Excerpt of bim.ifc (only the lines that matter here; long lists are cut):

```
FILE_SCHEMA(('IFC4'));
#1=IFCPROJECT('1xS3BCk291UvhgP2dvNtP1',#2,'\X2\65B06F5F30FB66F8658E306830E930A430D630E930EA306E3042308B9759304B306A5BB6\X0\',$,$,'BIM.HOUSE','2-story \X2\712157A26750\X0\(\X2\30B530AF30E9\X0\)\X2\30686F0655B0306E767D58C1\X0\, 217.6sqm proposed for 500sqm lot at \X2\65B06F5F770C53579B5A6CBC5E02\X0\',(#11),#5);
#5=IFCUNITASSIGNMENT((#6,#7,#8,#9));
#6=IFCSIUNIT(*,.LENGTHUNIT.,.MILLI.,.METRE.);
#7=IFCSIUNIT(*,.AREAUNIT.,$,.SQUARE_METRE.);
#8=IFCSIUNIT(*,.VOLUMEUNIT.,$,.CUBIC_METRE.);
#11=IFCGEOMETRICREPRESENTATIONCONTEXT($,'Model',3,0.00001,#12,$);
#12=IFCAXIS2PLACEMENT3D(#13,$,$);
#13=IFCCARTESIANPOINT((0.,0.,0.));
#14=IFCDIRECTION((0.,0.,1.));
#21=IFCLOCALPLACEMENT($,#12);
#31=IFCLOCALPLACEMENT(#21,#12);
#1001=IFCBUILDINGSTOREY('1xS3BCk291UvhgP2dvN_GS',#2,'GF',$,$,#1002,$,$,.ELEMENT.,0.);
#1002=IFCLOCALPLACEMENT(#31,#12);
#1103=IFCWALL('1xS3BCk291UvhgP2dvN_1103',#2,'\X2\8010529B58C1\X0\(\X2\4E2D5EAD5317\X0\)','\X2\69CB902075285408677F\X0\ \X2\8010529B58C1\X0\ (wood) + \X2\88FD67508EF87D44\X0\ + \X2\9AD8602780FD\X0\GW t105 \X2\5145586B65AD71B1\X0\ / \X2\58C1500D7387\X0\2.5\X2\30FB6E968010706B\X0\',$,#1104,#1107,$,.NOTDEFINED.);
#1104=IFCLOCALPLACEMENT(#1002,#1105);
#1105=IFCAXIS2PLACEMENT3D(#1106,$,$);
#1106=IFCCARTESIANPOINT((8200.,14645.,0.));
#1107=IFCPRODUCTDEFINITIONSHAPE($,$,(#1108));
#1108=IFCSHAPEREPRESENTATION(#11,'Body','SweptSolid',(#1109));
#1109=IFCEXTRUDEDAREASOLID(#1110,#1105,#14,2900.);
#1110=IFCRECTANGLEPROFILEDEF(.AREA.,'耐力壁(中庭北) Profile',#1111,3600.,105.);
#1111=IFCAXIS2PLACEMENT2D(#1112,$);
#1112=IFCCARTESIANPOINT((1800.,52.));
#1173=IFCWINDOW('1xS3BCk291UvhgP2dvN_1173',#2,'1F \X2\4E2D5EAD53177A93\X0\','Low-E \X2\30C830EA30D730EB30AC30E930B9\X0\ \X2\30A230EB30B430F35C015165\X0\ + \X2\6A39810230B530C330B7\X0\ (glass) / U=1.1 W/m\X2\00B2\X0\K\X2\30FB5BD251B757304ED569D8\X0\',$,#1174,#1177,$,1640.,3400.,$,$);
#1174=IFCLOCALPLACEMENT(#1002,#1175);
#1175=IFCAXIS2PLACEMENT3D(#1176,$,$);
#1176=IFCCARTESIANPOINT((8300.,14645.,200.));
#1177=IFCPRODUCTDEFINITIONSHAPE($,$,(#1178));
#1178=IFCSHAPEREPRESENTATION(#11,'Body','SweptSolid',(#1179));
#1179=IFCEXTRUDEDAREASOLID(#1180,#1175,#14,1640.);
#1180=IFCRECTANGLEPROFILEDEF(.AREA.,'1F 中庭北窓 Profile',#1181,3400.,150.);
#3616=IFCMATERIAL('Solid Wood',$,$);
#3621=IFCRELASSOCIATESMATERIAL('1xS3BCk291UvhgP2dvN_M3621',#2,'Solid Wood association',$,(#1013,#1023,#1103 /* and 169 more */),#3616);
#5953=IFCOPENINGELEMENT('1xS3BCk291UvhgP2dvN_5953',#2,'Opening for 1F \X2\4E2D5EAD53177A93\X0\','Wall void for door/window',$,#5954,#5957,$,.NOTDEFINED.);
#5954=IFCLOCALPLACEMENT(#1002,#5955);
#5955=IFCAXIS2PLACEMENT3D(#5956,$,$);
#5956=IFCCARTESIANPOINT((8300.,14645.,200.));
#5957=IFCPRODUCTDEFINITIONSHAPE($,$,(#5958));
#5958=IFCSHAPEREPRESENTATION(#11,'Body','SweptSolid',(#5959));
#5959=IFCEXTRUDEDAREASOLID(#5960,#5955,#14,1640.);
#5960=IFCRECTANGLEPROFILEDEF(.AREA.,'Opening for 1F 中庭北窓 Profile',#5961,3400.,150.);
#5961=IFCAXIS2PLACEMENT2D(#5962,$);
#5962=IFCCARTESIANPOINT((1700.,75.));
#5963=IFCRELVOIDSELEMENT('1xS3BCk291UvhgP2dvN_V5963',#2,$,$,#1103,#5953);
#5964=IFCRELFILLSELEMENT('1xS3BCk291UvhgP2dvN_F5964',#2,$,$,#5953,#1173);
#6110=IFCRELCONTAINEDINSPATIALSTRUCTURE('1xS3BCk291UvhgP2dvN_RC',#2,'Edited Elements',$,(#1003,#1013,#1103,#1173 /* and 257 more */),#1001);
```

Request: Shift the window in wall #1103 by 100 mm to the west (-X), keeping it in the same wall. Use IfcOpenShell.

```python
import ifcopenshell
import ifcopenshell.api.geometry
import ifcopenshell.util.placement
import ifcopenshell.util.unit

model = ifcopenshell.open("bim.ifc")
unit_scale = ifcopenshell.util.unit.calculate_unit_scale(model)

window = model.by_id(1173)
opening = window.FillsVoids[0].RelatingOpeningElement
wall = opening.VoidsElements[0].RelatingBuildingElement

wall_matrix = ifcopenshell.util.placement.get_local_placement(wall.ObjectPlacement)
shift = wall_matrix[:3, 0] * -0.1 / unit_scale
before = ifcopenshell.util.placement.get_local_placement(window.ObjectPlacement)[:3, 3].copy()

# The window is not placed relative to its opening, so move both.
for product in (opening, window):
    matrix = ifcopenshell.util.placement.get_local_placement(product.ObjectPlacement)
    matrix[:3, 3] += shift
    ifcopenshell.api.geometry.edit_object_placement(model, product=product, matrix=matrix, is_si=False)

after = ifcopenshell.util.placement.get_local_placement(window.ObjectPlacement)[:3, 3]
print("window moved by", (after - before).round(3) + 0.0)

model.write("bim_v2.ifc")
```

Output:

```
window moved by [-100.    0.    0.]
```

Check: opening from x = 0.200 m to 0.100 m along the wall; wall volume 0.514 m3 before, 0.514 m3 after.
